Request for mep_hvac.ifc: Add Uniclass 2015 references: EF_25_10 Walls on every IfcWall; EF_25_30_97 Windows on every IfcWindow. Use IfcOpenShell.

First a look at what the model holds.

```python
import ifcopenshell

model = ifcopenshell.open("mep_hvac.ifc")
print(model.schema)
print("classifications:", [c.Name for c in model.by_type("IfcClassification")])
for ifc_class in ("IfcDoor", "IfcRoof", "IfcStair", "IfcWall", "IfcWindow"):
    print(ifc_class, len(model.by_type(ifc_class)))
```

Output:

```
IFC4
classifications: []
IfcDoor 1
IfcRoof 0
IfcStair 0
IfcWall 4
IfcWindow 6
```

```python
import ifcopenshell
import ifcopenshell.api.classification

model = ifcopenshell.open("mep_hvac.ifc")

system = ifcopenshell.api.classification.add_classification(model, classification="Uniclass 2015")

codes = {
    "IfcWall": ("EF_25_10", "Walls"),
    "IfcWindow": ("EF_25_30_97", "Windows"),
}
for ifc_class, (code, name) in codes.items():
    products = model.by_type(ifc_class)
    ifcopenshell.api.classification.add_reference(
        model, products=products, classification=system, identification=code, name=name
    )
    print(code, len(products))

model.write("mep_hvac-out.ifc")
```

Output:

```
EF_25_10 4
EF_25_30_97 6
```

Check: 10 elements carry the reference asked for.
